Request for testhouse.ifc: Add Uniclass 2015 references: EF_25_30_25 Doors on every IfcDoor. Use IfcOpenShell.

First a look at what the model holds.

```python
import ifcopenshell

model = ifcopenshell.open("testhouse.ifc")
print(model.schema)
print("classifications:", [c.Name for c in model.by_type("IfcClassification")])
for ifc_class in ("IfcDoor", "IfcRoof", "IfcStair", "IfcWall", "IfcWindow"):
    print(ifc_class, len(model.by_type(ifc_class)))
```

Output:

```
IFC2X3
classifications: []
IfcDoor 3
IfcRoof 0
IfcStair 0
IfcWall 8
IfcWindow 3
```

```python
import ifcopenshell
import ifcopenshell.api.classification

model = ifcopenshell.open("testhouse.ifc")

# IFC2X3 requires Source and Edition and has no link from the project to the system.
system = model.create_entity("IfcClassification", Source="NBS", Edition="2015", Name="Uniclass 2015")

codes = {
    "IfcDoor": ("EF_25_30_25", "Doors"),
}
for ifc_class, (code, name) in codes.items():
    products = model.by_type(ifc_class)
    ifcopenshell.api.classification.add_reference(
        model, products=products, classification=system, identification=code, name=name
    )
    print(code, len(products))

model.write("testhouse_updated.ifc")
```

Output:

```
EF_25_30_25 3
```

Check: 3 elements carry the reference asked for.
